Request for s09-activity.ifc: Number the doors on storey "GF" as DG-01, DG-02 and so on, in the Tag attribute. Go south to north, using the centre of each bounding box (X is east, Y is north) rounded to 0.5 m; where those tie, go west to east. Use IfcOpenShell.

First a look at what the model holds.

```python
import ifcopenshell
import ifcopenshell.util.element
import ifcopenshell.util.placement

model = ifcopenshell.open("s09-activity.ifc")
print(model.schema)
storey = next(s for s in model.by_type("IfcBuildingStorey") if s.Name == "GF")
doors = [e for e in ifcopenshell.util.element.get_decomposition(storey) if e.is_a("IfcDoor")]
for e in sorted(doors, key=lambda e: e.id()):
    origin = ifcopenshell.util.placement.get_local_placement(e.ObjectPlacement)[:3, 3]
    print(e.id(), e.Tag, e.Name, origin.round(2) + 0.0, sep=" | ")
```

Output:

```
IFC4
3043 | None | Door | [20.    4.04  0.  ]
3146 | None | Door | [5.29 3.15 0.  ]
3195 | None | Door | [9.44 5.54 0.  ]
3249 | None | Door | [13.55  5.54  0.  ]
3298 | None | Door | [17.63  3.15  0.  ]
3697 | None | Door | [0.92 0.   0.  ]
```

```python
import ifcopenshell
import ifcopenshell.geom
import ifcopenshell.util.element
import ifcopenshell.util.shape

model = ifcopenshell.open("s09-activity.ifc")
settings = ifcopenshell.geom.settings()
settings.set("use-world-coords", True)


def centre(element):
    shape = ifcopenshell.geom.create_shape(settings, element)
    return ifcopenshell.util.shape.get_bbox_centroid(shape.geometry)


storey = next(s for s in model.by_type("IfcBuildingStorey") if s.Name == "GF")
doors = [e for e in ifcopenshell.util.element.get_decomposition(storey) if e.is_a("IfcDoor")]

# Insertion points can sit at a corner or the storey origin, so sort by the geometry (in metres).
centres = {e: centre(e) for e in doors}
doors.sort(key=lambda e: (round(centres[e][1] / 0.5), centres[e][0]))

for i, e in enumerate(doors, start=1):
    number = f"DG-{i:02d}"
    e.Tag = number
    print(e.id(), number)

model.write("s09-activity_edited.ifc")
```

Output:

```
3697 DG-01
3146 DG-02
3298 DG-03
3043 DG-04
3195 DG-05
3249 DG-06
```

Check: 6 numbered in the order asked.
